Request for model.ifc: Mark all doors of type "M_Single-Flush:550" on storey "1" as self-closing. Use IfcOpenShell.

First a look at what the model holds.

```python
import ifcopenshell
import ifcopenshell.util.element

model = ifcopenshell.open("model.ifc")
print(model.schema)
storey = next(s for s in model.by_type("IfcBuildingStorey") if s.Name == "1")
doors = [e for e in ifcopenshell.util.element.get_decomposition(storey) if e.is_a("IfcDoor")]
seen = {}
for e in doors:
    element_type = ifcopenshell.util.element.get_type(e)
    key = (element_type.Name if element_type != e and element_type else None, ifcopenshell.util.element.get_pset(e, "Pset_DoorCommon", "SelfClosing"))
    seen[key] = seen.get(key, 0) + 1
for (name, value), count in sorted(seen.items(), key=str):
    print(count, "x", name, "|", value)
```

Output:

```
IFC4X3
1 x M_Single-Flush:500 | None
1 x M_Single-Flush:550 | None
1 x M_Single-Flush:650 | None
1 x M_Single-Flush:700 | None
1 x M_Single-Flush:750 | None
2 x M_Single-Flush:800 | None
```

```python
import ifcopenshell
import ifcopenshell.api.pset
import ifcopenshell.util.element

model = ifcopenshell.open("model.ifc")

storey = next(s for s in model.by_type("IfcBuildingStorey") if s.Name == "1")
doors = [e for e in ifcopenshell.util.element.get_decomposition(storey) if e.is_a("IfcDoor")]

count = 0
for e in doors:
    element_type = ifcopenshell.util.element.get_type(e)
    if element_type in (None, e) or element_type.Name != "M_Single-Flush:550":
        continue
    # add_pset returns the element's existing set when there is one.
    pset = ifcopenshell.api.pset.add_pset(model, product=e, name="Pset_DoorCommon")
    ifcopenshell.api.pset.edit_pset(model, pset=pset, properties={"SelfClosing": True})
    count += 1

print(count, "doors updated")

model.write("model_v2.ifc")
```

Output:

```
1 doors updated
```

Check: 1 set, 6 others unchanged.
